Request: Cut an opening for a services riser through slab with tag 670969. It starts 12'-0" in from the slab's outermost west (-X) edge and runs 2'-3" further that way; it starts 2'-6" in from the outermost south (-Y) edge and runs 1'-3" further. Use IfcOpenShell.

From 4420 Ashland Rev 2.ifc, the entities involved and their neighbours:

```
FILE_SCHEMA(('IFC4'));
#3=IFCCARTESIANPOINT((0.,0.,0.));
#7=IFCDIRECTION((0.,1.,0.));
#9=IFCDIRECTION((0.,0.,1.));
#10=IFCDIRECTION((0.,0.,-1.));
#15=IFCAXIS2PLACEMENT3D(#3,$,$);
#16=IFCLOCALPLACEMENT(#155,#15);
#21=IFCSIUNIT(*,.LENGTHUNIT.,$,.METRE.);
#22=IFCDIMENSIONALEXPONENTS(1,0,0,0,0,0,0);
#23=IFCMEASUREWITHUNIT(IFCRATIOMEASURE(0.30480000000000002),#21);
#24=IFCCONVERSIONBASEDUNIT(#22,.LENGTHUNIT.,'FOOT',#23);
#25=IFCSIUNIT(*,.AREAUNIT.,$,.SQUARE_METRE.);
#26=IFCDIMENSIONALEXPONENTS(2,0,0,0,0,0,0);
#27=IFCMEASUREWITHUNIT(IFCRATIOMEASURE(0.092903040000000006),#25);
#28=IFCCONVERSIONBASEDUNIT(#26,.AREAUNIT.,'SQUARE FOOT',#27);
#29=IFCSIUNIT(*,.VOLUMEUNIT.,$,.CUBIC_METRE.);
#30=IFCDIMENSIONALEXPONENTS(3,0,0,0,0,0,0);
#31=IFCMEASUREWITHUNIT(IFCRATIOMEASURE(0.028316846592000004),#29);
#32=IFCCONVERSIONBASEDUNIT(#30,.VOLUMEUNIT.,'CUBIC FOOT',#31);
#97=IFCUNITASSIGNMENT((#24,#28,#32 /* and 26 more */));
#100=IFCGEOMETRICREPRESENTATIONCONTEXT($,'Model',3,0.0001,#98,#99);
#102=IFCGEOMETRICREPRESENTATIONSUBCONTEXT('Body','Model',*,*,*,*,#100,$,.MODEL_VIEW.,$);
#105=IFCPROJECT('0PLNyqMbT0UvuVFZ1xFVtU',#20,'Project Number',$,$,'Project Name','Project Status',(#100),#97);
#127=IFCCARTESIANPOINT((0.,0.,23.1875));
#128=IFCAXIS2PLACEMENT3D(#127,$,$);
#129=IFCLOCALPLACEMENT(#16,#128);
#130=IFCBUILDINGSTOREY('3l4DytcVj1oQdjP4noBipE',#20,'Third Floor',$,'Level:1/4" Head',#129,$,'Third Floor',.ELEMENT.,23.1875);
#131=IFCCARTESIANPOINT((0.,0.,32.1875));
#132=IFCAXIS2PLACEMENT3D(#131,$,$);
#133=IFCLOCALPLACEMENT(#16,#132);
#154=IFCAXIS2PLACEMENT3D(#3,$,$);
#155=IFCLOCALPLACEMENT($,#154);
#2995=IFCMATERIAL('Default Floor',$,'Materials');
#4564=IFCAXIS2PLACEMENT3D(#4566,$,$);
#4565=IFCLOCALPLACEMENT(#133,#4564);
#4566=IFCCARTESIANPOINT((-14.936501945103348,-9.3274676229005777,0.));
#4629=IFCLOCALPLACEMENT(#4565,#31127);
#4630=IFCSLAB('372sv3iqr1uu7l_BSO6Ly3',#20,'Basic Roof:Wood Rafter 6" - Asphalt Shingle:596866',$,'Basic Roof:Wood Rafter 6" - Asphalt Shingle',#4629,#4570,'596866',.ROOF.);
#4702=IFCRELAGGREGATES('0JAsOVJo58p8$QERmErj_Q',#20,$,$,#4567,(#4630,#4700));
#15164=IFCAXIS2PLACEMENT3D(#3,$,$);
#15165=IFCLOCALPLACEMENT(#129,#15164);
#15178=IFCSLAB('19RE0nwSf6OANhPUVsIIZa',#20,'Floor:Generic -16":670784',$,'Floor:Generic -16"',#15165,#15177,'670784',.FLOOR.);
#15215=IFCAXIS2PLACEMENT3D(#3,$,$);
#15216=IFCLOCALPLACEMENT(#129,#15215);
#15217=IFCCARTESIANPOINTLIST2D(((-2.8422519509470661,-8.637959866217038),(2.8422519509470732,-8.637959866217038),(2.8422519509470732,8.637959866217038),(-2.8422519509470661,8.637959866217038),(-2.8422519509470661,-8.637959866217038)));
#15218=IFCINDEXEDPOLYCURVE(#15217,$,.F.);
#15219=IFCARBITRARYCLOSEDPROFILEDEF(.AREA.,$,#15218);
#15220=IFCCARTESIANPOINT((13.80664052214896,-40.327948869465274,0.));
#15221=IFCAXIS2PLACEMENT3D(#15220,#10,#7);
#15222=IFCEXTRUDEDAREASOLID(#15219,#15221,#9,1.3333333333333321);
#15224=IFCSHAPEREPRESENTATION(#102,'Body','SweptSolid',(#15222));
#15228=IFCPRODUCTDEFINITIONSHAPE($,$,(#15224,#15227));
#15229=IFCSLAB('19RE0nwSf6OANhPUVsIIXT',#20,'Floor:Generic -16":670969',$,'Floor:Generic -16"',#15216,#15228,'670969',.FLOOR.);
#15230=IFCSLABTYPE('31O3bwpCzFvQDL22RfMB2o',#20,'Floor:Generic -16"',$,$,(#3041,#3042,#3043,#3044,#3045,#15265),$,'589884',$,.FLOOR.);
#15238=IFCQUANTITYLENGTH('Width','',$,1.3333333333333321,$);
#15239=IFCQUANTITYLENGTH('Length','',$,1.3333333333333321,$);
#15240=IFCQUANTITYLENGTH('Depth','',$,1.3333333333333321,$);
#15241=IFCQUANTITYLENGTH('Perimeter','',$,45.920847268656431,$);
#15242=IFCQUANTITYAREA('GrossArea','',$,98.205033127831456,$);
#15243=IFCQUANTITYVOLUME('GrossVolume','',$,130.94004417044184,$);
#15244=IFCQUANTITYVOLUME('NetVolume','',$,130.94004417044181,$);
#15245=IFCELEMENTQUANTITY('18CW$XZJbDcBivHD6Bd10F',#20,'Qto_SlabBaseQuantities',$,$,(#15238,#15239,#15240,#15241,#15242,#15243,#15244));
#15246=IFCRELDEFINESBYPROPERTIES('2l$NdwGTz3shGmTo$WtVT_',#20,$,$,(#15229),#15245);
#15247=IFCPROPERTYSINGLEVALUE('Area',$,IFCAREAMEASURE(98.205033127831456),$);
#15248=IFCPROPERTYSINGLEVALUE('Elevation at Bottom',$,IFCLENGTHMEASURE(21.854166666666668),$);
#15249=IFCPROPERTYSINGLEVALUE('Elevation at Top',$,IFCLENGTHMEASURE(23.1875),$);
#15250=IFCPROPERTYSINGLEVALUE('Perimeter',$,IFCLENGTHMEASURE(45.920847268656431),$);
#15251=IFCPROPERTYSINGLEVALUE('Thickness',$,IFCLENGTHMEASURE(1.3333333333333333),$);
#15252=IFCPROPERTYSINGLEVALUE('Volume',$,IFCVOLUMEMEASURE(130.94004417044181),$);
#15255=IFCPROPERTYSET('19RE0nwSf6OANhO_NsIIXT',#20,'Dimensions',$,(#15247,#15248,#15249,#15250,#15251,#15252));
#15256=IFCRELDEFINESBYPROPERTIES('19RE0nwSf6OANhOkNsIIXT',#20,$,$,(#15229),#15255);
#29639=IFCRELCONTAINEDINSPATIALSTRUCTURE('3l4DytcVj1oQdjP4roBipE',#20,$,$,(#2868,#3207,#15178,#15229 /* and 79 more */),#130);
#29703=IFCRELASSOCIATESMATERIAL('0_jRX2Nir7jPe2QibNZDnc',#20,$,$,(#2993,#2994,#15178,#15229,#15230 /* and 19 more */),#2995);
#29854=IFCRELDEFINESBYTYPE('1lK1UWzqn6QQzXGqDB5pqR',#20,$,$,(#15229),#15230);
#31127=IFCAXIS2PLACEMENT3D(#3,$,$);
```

```python
import numpy as np
import ifcopenshell
import ifcopenshell.api.feature
import ifcopenshell.api.geometry
import ifcopenshell.api.pset
import ifcopenshell.api.root
import ifcopenshell.geom
import ifcopenshell.util.element
import ifcopenshell.util.placement
import ifcopenshell.util.representation
import ifcopenshell.util.shape
import ifcopenshell.util.unit

model = ifcopenshell.open("4420 Ashland Rev 2.ifc")
unit_scale = ifcopenshell.util.unit.calculate_unit_scale(model)
area_scale = ifcopenshell.util.unit.calculate_unit_scale(model, "AREAUNIT")
volume_scale = ifcopenshell.util.unit.calculate_unit_scale(model, "VOLUMEUNIT")
settings = ifcopenshell.geom.settings()


def volume(element):
    """Net volume in cubic metres, openings subtracted."""
    shape = ifcopenshell.geom.create_shape(settings, element)
    return ifcopenshell.util.shape.get_volume(shape.geometry)


slab = model.by_guid("19RE0nwSf6OANhPUVsIIXT")
before = volume(slab)

# Extent in the slab's own axes, in metres. The edges named are its -X and -Y sides.
slab_shape = ifcopenshell.geom.create_shape(settings, slab)
vertices = ifcopenshell.util.shape.get_vertices(slab_shape.geometry)
x_min, y_min, bottom = vertices.min(axis=0)
top = vertices[:, 2].max()

opening = ifcopenshell.api.root.create_entity(model, ifc_class="IfcOpeningElement", name="Services riser opening", predefined_type="OPENING")
context = ifcopenshell.util.representation.get_context(model, "Model", "Body", "MODEL_VIEW")
width, depth = 0.6858, 0.381
outline = [(0.0, 0.0), (width, 0.0), (width, depth), (0.0, depth), (0.0, 0.0)]
# Overshoot both faces by 50 mm so the cut is clean.
shape = ifcopenshell.api.geometry.add_slab_representation(
    model, context=context, depth=top - bottom + 0.1, polyline=outline
)
ifcopenshell.api.geometry.assign_representation(model, product=opening, representation=shape)

matrix = ifcopenshell.util.placement.get_local_placement(slab.ObjectPlacement)
matrix[:, 3] = matrix @ np.append(np.array([x_min + 3.6576, y_min + 0.762, bottom - 0.05]) / unit_scale, 1.0)
ifcopenshell.api.geometry.edit_object_placement(model, product=opening, matrix=matrix, is_si=False)
ifcopenshell.api.feature.add_feature(model, feature=opening, element=slab)

after = volume(slab)

# Update the slab's stored quantities.
qto = model.by_id(ifcopenshell.util.element.get_pset(slab, "Qto_SlabBaseQuantities", should_inherit=False)["id"])
ifcopenshell.api.pset.edit_qto(model, qto=qto, properties={"NetVolume": after / volume_scale})
pset = model.by_id(ifcopenshell.util.element.get_pset(slab, "Dimensions", should_inherit=False)["id"])
ifcopenshell.api.pset.edit_pset(model, pset=pset, properties={
    "Area": model.create_entity("IfcAreaMeasure", after / (top - bottom) / area_scale),
    "Volume": model.create_entity("IfcVolumeMeasure", after / volume_scale),
})

print(f"slab volume {before:.3f} -> {after:.3f} m3")

model.write("4420 Ashland Rev 2_v2.ifc")
```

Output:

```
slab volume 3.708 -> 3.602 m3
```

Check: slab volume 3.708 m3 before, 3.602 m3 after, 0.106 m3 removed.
